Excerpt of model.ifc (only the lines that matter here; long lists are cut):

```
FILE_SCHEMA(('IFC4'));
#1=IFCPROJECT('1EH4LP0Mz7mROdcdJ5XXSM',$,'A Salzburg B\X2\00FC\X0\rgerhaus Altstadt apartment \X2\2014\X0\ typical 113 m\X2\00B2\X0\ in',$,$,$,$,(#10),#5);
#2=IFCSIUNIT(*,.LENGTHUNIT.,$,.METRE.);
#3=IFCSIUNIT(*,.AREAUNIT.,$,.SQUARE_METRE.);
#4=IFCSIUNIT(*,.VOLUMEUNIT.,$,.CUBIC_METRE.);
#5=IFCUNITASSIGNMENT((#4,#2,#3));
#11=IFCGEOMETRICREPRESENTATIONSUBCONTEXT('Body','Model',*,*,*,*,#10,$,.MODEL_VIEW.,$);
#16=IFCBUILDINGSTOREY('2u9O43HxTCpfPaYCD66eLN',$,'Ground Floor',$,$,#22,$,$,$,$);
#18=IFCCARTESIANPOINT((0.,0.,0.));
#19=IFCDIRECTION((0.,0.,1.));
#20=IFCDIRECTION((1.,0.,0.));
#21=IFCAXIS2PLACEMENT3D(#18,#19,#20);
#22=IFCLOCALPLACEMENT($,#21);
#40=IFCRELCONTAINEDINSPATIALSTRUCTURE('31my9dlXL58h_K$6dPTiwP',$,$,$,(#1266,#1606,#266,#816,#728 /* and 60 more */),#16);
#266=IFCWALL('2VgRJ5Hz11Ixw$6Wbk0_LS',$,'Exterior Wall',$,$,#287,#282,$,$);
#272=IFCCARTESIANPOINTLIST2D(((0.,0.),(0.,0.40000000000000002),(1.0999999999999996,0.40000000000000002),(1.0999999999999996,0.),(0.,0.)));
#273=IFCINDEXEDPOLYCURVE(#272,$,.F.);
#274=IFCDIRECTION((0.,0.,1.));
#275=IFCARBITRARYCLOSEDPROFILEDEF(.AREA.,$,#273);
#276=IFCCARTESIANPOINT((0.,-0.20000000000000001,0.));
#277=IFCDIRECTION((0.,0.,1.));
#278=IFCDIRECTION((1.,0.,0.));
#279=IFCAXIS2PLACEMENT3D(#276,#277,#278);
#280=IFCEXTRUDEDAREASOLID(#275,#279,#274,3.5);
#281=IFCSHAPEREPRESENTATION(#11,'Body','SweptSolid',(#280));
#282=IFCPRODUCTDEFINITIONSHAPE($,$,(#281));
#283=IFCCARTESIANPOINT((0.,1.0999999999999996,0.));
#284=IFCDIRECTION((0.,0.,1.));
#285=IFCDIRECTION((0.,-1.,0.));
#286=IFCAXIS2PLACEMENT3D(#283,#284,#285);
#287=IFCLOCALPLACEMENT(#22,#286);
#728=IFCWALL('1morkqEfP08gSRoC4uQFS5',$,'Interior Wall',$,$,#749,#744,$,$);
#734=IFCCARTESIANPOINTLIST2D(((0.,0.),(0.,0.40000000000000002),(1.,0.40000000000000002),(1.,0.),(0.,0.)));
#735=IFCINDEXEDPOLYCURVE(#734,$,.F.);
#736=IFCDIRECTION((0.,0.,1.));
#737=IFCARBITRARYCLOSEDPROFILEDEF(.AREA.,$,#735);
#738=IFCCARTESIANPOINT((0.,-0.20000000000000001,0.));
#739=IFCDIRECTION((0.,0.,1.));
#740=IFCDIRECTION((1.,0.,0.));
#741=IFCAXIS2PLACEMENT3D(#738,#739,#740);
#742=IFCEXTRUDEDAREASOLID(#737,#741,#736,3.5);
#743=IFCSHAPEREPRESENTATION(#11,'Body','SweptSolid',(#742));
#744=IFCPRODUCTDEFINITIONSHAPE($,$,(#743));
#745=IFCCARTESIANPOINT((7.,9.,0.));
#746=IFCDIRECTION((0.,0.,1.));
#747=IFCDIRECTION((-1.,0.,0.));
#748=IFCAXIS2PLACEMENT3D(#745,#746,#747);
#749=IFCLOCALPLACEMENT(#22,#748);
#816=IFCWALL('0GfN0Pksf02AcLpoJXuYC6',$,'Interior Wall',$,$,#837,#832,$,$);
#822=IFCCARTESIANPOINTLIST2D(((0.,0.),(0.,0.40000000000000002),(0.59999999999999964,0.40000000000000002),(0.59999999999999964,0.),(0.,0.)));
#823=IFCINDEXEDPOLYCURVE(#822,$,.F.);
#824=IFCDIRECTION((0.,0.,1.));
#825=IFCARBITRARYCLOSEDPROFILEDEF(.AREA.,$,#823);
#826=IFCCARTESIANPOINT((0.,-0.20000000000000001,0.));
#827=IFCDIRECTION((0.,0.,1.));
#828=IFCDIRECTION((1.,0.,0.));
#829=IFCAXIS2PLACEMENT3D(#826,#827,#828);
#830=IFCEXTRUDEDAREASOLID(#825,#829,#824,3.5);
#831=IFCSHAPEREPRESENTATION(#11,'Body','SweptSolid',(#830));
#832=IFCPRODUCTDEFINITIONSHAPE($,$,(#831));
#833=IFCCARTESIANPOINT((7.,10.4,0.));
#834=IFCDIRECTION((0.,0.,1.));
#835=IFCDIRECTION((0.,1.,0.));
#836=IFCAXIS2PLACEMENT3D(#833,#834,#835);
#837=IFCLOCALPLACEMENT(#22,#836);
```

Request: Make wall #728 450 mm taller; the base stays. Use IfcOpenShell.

```python
import ifcopenshell
import ifcopenshell.geom
import ifcopenshell.util.representation
import ifcopenshell.util.shape
import ifcopenshell.util.unit

model = ifcopenshell.open("model.ifc")
unit_scale = ifcopenshell.util.unit.calculate_unit_scale(model)
settings = ifcopenshell.geom.settings()


def volume(element):
    """Net volume in cubic metres, openings subtracted."""
    shape = ifcopenshell.geom.create_shape(settings, element)
    return ifcopenshell.util.shape.get_volume(shape.geometry)


wall = model.by_id(728)
before = volume(wall)

body = ifcopenshell.util.representation.get_representation(wall, "Model", "Body")
solid = body.Items[0]
old_height = solid.Depth
solid.Depth += 0.45 / unit_scale
after = volume(wall)

print(f"height {old_height:g} -> {solid.Depth:g}, volume {before:.3f} -> {after:.3f} m3")

model.write("model_edited.ifc")
```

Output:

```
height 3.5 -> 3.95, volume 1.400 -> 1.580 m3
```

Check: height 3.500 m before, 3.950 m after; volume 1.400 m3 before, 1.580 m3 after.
